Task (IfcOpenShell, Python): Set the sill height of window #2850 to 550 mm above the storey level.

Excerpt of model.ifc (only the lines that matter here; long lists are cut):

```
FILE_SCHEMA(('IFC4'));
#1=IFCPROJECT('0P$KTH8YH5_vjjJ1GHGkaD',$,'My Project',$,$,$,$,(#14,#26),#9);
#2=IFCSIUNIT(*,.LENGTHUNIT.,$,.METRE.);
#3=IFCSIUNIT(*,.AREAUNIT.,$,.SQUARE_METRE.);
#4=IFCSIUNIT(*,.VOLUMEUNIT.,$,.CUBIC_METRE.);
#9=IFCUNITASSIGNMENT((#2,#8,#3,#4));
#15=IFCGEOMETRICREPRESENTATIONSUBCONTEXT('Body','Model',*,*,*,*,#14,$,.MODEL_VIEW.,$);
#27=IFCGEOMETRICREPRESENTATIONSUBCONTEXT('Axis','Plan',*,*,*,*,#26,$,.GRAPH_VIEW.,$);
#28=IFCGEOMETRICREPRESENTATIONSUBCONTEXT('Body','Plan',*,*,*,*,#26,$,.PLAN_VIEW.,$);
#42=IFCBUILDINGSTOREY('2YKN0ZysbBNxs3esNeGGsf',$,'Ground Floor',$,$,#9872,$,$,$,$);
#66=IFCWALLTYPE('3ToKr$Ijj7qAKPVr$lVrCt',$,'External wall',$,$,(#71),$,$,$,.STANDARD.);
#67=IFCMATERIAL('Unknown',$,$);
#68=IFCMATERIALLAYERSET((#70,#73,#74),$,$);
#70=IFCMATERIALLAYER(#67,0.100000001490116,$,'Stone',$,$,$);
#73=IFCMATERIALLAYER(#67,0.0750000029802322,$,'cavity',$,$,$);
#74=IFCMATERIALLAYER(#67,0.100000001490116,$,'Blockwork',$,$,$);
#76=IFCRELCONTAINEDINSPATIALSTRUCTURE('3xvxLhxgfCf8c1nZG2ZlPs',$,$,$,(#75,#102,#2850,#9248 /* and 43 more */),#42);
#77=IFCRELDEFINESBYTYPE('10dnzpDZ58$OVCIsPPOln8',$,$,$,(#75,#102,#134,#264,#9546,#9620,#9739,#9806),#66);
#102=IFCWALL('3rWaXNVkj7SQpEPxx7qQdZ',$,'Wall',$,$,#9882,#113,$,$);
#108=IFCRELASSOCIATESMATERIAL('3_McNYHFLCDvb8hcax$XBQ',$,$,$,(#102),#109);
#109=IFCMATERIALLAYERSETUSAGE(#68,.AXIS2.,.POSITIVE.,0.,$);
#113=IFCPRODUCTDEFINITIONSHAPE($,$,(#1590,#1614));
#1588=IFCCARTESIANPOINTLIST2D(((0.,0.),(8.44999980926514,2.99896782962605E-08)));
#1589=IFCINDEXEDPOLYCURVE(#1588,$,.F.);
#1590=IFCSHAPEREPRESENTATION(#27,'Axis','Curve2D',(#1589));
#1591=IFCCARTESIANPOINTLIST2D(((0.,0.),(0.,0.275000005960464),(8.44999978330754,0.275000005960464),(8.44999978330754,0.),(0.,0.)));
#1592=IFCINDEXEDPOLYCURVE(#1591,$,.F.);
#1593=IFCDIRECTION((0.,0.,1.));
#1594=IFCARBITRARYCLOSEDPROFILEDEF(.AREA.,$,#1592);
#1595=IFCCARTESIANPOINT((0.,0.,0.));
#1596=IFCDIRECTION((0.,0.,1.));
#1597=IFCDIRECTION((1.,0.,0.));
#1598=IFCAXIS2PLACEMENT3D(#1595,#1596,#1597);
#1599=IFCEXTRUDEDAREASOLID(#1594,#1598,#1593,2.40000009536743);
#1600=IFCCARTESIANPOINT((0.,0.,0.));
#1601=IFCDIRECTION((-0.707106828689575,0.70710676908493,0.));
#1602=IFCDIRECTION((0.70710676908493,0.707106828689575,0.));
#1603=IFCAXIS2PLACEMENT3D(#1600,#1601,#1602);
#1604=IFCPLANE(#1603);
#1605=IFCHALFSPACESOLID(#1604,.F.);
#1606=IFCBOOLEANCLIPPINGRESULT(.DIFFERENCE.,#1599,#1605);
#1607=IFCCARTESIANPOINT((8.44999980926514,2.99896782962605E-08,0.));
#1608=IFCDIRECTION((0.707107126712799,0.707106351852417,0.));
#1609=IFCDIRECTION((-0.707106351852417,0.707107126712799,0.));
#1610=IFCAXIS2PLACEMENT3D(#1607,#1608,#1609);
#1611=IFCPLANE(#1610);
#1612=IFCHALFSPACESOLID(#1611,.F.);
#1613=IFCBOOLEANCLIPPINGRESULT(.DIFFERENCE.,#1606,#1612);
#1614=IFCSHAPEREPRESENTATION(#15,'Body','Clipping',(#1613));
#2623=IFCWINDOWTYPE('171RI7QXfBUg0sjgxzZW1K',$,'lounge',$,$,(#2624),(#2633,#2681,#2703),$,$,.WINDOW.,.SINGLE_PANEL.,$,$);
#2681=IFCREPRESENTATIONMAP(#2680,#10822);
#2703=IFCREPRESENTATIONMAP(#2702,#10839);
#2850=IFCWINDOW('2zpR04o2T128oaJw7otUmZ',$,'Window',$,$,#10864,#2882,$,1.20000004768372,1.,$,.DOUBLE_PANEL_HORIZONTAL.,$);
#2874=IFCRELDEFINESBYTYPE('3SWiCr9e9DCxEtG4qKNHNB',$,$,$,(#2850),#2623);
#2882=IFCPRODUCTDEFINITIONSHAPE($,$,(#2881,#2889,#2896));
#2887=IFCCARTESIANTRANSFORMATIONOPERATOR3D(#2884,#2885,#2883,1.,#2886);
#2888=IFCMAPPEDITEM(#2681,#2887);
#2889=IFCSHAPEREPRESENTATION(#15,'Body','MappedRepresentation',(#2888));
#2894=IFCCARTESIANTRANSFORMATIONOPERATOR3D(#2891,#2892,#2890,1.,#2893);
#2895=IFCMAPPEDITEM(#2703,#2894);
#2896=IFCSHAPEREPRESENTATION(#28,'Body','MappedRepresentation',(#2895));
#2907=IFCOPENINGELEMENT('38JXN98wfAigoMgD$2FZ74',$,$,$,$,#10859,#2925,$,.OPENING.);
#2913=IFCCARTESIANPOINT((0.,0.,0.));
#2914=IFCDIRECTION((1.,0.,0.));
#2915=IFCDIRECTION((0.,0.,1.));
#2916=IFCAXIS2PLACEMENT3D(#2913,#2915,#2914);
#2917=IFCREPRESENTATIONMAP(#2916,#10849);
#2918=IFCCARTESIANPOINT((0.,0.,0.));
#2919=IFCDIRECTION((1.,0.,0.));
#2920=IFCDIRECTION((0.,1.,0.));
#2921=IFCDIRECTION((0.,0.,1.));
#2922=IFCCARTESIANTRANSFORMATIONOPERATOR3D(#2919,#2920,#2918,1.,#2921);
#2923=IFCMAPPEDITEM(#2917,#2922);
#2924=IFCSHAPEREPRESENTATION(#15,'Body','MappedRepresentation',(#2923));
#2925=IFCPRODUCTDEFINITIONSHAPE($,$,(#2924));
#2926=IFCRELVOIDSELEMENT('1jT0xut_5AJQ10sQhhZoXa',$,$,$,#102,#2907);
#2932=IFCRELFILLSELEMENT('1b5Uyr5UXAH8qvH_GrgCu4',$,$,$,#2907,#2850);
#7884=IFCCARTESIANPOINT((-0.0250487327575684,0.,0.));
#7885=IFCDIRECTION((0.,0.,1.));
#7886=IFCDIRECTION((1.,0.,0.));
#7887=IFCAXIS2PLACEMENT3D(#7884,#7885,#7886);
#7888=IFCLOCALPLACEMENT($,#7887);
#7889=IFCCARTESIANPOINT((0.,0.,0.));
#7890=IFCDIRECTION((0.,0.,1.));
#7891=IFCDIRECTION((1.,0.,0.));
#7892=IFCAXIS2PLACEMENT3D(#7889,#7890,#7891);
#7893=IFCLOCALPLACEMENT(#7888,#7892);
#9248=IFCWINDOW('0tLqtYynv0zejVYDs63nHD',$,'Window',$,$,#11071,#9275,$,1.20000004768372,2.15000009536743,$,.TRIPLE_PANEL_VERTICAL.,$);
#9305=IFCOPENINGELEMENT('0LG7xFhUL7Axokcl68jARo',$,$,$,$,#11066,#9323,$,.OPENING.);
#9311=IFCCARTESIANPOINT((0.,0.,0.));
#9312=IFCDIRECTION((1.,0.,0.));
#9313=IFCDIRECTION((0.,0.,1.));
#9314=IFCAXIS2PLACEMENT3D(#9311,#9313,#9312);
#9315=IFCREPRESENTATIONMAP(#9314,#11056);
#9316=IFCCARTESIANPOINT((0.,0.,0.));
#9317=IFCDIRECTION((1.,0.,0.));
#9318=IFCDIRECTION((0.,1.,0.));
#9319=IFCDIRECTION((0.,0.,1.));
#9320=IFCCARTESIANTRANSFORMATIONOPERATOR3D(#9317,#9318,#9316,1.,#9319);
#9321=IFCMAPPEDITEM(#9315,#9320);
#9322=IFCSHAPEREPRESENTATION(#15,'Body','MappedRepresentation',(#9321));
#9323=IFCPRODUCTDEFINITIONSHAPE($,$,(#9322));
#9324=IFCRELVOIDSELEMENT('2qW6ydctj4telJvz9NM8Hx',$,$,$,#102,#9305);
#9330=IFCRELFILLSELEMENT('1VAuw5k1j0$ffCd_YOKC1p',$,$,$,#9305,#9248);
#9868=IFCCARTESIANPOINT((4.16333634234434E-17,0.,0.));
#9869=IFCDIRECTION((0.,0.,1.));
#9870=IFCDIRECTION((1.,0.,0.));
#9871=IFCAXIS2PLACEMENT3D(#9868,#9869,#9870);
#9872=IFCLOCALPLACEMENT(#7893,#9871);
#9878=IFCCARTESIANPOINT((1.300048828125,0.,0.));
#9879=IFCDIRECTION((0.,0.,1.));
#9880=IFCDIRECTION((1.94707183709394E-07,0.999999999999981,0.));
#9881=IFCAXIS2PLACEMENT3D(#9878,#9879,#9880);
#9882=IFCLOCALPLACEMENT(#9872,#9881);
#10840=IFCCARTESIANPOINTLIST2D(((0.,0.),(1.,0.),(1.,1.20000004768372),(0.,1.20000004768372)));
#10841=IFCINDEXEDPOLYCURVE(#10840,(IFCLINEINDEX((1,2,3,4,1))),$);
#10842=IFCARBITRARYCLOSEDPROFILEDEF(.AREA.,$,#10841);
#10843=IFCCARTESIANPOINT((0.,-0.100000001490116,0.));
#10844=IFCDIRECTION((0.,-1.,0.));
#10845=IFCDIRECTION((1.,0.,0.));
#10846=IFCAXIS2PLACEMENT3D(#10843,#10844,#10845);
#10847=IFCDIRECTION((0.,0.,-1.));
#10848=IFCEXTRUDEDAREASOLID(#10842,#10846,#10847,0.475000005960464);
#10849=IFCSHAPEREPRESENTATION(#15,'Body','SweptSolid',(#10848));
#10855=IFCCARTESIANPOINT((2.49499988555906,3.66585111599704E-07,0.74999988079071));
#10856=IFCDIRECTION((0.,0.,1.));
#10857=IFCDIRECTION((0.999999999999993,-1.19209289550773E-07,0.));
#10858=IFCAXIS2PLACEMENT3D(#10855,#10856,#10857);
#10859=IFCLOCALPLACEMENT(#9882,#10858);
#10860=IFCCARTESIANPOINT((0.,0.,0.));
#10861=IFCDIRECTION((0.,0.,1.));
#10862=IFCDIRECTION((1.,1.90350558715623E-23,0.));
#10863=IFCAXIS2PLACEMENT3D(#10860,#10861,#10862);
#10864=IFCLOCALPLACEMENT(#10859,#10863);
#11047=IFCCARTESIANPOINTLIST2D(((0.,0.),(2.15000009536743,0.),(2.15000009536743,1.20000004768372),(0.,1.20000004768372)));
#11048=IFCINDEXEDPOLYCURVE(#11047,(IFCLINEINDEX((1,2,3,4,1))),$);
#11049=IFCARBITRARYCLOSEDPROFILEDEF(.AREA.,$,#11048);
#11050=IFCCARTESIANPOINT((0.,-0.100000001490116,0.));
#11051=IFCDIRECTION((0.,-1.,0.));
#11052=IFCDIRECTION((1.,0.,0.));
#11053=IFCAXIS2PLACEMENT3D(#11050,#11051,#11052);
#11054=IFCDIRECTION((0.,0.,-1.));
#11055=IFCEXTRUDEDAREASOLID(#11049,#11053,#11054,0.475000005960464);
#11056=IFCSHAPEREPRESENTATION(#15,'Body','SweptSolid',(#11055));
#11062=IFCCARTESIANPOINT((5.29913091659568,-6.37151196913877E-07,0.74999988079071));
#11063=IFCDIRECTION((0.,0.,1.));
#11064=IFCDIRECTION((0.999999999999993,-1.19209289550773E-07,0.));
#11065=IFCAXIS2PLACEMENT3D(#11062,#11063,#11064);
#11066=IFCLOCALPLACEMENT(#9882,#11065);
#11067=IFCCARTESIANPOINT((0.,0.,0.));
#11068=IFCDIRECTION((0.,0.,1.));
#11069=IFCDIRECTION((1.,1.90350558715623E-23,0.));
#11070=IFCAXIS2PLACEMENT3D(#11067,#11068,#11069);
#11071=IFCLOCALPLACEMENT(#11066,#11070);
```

```python
import numpy as np
import ifcopenshell
import ifcopenshell.api.geometry
import ifcopenshell.geom
import ifcopenshell.util.element
import ifcopenshell.util.placement
import ifcopenshell.util.shape
import ifcopenshell.util.unit

model = ifcopenshell.open("model.ifc")
unit_scale = ifcopenshell.util.unit.calculate_unit_scale(model)

window = model.by_guid("2zpR04o2T128oaJw7otUmZ")
opening = window.FillsVoids[0].RelatingOpeningElement
storey = ifcopenshell.util.element.get_container(window, ifc_class="IfcBuildingStorey")
level = ifcopenshell.util.placement.get_local_placement(storey.ObjectPlacement)[2, 3]

# The opening's origin need not be at the sill, so measure its lowest point.
shape = ifcopenshell.geom.create_shape(ifcopenshell.geom.settings(), opening)
bottom = ifcopenshell.util.shape.get_shape_bottom_elevation(shape, shape.geometry) / unit_scale
dz = level + 0.55 - bottom

shift = np.array([0.0, 0.0, dz])
# The window is placed relative to its opening, so it follows when the opening moves.
matrix = ifcopenshell.util.placement.get_local_placement(opening.ObjectPlacement)
matrix[:3, 3] += shift
ifcopenshell.api.geometry.edit_object_placement(
    model, product=opening, matrix=matrix, is_si=False, should_transform_children=True
)

print(f"moved by {dz * unit_scale:+.3f} m")

model.write("model_edited.ifc")
```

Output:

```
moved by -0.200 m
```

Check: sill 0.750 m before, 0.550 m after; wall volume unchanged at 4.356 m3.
